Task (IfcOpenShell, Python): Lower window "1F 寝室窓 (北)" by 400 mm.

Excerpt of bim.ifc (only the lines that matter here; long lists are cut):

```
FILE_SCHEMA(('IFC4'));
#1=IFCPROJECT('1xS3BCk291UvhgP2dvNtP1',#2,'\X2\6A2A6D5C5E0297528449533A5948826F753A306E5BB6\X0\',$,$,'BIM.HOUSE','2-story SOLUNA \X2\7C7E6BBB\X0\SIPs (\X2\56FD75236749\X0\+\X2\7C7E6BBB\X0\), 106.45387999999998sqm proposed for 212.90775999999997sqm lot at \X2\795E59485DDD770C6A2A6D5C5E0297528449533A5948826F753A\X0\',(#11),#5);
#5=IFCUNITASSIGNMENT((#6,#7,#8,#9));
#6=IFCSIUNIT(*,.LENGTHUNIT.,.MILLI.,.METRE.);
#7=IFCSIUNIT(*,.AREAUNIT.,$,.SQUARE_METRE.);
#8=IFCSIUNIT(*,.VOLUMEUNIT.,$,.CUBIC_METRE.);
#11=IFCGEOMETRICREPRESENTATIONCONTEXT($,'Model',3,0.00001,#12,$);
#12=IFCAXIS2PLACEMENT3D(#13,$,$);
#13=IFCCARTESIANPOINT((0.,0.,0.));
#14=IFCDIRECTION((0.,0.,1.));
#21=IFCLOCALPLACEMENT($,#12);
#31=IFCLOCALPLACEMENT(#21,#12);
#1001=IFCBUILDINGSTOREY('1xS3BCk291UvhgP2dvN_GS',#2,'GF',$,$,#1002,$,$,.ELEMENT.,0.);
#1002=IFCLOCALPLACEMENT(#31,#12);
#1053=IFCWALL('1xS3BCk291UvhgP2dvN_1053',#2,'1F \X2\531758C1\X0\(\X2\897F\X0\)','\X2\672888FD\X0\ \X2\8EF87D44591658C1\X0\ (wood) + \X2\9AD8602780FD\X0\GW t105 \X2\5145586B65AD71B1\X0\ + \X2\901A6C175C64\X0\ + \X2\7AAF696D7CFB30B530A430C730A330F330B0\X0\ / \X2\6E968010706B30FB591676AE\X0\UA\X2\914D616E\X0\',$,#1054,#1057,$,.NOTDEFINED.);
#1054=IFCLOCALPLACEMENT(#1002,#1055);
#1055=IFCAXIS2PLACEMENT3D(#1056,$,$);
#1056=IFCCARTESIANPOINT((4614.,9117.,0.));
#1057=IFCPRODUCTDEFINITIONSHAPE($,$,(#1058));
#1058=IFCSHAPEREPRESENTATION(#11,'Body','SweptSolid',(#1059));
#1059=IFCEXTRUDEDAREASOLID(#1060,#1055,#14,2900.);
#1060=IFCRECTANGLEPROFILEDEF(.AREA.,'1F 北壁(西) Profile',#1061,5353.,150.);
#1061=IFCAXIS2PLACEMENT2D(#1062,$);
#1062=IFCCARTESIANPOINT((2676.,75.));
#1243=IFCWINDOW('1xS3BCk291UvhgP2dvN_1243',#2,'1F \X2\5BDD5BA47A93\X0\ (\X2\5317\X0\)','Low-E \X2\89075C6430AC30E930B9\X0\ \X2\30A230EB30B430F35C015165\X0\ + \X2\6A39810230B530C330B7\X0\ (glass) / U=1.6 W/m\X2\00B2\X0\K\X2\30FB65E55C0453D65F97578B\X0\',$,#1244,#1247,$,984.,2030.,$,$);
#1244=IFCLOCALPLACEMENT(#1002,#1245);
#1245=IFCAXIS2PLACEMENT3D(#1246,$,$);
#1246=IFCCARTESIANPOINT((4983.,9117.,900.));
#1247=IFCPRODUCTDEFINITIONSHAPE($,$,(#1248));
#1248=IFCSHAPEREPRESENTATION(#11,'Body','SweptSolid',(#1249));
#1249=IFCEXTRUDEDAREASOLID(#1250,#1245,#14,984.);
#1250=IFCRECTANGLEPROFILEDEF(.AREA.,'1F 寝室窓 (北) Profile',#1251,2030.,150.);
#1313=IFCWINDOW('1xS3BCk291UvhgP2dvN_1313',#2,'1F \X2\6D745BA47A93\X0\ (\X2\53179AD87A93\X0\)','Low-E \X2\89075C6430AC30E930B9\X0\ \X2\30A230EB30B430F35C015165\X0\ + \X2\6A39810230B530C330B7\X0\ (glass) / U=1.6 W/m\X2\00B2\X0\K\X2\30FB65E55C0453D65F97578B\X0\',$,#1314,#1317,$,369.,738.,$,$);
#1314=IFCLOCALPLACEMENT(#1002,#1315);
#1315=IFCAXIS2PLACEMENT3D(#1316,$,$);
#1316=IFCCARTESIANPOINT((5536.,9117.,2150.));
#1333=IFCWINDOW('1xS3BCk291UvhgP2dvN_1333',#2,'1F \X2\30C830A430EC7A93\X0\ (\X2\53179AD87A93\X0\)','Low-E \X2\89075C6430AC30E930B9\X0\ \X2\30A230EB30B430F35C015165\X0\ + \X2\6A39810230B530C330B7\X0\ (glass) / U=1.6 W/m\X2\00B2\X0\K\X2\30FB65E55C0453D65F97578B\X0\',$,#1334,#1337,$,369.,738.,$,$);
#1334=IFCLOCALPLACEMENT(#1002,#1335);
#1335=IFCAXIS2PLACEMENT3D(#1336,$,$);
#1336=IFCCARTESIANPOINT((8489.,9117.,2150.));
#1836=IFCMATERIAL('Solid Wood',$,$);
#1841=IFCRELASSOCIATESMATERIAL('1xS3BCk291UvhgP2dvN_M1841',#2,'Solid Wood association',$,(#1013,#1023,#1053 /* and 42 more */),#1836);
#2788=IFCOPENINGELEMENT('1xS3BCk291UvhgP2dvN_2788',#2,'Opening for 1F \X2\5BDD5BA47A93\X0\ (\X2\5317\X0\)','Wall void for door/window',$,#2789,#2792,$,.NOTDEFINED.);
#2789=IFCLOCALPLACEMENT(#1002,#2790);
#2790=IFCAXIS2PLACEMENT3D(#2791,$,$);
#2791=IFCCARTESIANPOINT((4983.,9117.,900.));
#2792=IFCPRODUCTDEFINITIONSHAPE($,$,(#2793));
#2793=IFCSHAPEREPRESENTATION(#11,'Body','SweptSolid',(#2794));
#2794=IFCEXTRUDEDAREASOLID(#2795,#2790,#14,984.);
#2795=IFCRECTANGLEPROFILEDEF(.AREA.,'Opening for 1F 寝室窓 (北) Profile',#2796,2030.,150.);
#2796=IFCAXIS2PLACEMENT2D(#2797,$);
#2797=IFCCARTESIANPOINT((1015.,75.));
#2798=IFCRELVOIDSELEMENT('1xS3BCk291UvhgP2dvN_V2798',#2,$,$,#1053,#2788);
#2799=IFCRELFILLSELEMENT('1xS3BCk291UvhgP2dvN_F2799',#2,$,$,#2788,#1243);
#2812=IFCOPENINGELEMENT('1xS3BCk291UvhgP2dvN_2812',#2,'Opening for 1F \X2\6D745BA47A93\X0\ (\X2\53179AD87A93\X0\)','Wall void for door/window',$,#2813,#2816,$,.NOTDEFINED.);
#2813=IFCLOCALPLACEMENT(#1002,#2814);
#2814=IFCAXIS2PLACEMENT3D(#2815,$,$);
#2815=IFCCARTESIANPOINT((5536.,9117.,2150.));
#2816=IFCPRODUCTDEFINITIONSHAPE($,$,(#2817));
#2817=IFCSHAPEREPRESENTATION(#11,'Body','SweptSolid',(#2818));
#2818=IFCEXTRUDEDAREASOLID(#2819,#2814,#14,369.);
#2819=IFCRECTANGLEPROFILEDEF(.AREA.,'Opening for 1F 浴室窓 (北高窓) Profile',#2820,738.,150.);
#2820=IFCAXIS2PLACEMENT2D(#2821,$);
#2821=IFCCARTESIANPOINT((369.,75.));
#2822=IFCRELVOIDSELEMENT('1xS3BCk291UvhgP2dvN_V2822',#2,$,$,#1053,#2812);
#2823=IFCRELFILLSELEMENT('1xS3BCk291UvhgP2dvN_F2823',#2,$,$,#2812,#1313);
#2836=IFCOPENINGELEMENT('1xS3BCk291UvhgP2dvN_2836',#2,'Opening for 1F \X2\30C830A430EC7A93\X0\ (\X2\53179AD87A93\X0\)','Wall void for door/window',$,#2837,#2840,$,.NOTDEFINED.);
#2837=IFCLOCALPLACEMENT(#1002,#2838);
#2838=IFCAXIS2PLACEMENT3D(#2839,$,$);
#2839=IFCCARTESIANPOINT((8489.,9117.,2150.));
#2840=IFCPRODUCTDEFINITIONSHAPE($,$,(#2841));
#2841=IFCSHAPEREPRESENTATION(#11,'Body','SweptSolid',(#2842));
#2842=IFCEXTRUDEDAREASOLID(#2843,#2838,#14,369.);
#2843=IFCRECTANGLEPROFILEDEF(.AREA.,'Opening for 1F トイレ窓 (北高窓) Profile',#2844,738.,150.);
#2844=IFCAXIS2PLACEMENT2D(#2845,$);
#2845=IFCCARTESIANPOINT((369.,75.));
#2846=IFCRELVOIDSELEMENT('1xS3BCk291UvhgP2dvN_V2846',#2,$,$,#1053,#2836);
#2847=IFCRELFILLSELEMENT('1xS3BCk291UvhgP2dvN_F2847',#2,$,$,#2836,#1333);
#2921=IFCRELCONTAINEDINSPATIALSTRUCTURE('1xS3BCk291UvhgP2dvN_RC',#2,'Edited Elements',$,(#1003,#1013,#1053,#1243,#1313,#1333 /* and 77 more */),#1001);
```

```python
import numpy as np
import ifcopenshell
import ifcopenshell.api.geometry
import ifcopenshell.util.placement
import ifcopenshell.util.unit

model = ifcopenshell.open("bim.ifc")
unit_scale = ifcopenshell.util.unit.calculate_unit_scale(model)

window = model.by_id(1243)
opening = window.FillsVoids[0].RelatingOpeningElement
dz = -0.4 / unit_scale

shift = np.array([0.0, 0.0, dz])
# The window is not placed relative to its opening, so move both.
for product in (opening, window):
    matrix = ifcopenshell.util.placement.get_local_placement(product.ObjectPlacement)
    matrix[:3, 3] += shift
    ifcopenshell.api.geometry.edit_object_placement(model, product=product, matrix=matrix, is_si=False)

print(f"moved by {dz * unit_scale:+.3f} m")

model.write("bim_v2.ifc")
```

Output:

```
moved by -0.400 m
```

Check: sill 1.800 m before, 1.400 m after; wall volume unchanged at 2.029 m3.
